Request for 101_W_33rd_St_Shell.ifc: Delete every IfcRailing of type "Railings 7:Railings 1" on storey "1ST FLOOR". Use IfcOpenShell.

First a look at what the model holds.

```python
import ifcopenshell
import ifcopenshell.util.element

model = ifcopenshell.open("101_W_33rd_St_Shell.ifc")
print(model.schema)
storey = next(s for s in model.by_type("IfcBuildingStorey") if s.Name == "1ST FLOOR")
railings = [e for e in ifcopenshell.util.element.get_decomposition(storey) if e.is_a("IfcRailing")]
seen = {}
for e in railings:
    element_type = ifcopenshell.util.element.get_type(e)
    name = element_type.Name if element_type not in (None, e) else None
    seen[name] = seen.get(name, 0) + 1
for name, count in sorted(seen.items(), key=str):
    print(count, "x", name)
```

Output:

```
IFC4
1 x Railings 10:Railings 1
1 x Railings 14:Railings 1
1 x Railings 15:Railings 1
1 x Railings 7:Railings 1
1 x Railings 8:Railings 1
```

```python
import ifcopenshell
import ifcopenshell.api.root
import ifcopenshell.util.element

model = ifcopenshell.open("101_W_33rd_St_Shell.ifc")

storey = next(s for s in model.by_type("IfcBuildingStorey") if s.Name == "1ST FLOOR")
railings = [e for e in ifcopenshell.util.element.get_decomposition(storey) if e.is_a("IfcRailing")]
targets = [e for e in railings if (t := ifcopenshell.util.element.get_type(e)) not in (None, e) and t.Name == "Railings 7:Railings 1"]

for e in targets:
    ifcopenshell.api.root.remove_product(model, product=e)
print(len(targets), "removed")

model.write("101_W_33rd_St_Shell_rev.ifc")
```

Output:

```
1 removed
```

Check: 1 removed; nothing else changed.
